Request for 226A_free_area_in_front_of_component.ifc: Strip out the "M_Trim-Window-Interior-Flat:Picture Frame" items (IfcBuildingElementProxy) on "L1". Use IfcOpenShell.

First a look at what the model holds.

```python
import ifcopenshell
import ifcopenshell.util.element

model = ifcopenshell.open("226A_free_area_in_front_of_component.ifc")
print(model.schema)
storey = next(s for s in model.by_type("IfcBuildingStorey") if s.Name == "L1")
proxies = [e for e in ifcopenshell.util.element.get_decomposition(storey) if e.is_a("IfcBuildingElementProxy")]
seen = {}
for e in proxies:
    element_type = ifcopenshell.util.element.get_type(e)
    name = element_type.Name if element_type not in (None, e) else None
    seen[name] = seen.get(name, 0) + 1
for name, count in sorted(seen.items(), key=str):
    print(count, "x", name)
```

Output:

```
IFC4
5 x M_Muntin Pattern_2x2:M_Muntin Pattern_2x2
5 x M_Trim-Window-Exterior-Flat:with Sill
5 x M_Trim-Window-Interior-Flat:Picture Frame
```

```python
import ifcopenshell
import ifcopenshell.api.root
import ifcopenshell.util.element

model = ifcopenshell.open("226A_free_area_in_front_of_component.ifc")

storey = next(s for s in model.by_type("IfcBuildingStorey") if s.Name == "L1")
proxies = [e for e in ifcopenshell.util.element.get_decomposition(storey) if e.is_a("IfcBuildingElementProxy")]
targets = [e for e in proxies if (t := ifcopenshell.util.element.get_type(e)) not in (None, e) and t.Name == "M_Trim-Window-Interior-Flat:Picture Frame"]

for e in targets:
    ifcopenshell.api.root.remove_product(model, product=e)
print(len(targets), "removed")

model.write("226A_free_area_in_front_of_component_edited.ifc")
```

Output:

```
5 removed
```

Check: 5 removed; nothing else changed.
